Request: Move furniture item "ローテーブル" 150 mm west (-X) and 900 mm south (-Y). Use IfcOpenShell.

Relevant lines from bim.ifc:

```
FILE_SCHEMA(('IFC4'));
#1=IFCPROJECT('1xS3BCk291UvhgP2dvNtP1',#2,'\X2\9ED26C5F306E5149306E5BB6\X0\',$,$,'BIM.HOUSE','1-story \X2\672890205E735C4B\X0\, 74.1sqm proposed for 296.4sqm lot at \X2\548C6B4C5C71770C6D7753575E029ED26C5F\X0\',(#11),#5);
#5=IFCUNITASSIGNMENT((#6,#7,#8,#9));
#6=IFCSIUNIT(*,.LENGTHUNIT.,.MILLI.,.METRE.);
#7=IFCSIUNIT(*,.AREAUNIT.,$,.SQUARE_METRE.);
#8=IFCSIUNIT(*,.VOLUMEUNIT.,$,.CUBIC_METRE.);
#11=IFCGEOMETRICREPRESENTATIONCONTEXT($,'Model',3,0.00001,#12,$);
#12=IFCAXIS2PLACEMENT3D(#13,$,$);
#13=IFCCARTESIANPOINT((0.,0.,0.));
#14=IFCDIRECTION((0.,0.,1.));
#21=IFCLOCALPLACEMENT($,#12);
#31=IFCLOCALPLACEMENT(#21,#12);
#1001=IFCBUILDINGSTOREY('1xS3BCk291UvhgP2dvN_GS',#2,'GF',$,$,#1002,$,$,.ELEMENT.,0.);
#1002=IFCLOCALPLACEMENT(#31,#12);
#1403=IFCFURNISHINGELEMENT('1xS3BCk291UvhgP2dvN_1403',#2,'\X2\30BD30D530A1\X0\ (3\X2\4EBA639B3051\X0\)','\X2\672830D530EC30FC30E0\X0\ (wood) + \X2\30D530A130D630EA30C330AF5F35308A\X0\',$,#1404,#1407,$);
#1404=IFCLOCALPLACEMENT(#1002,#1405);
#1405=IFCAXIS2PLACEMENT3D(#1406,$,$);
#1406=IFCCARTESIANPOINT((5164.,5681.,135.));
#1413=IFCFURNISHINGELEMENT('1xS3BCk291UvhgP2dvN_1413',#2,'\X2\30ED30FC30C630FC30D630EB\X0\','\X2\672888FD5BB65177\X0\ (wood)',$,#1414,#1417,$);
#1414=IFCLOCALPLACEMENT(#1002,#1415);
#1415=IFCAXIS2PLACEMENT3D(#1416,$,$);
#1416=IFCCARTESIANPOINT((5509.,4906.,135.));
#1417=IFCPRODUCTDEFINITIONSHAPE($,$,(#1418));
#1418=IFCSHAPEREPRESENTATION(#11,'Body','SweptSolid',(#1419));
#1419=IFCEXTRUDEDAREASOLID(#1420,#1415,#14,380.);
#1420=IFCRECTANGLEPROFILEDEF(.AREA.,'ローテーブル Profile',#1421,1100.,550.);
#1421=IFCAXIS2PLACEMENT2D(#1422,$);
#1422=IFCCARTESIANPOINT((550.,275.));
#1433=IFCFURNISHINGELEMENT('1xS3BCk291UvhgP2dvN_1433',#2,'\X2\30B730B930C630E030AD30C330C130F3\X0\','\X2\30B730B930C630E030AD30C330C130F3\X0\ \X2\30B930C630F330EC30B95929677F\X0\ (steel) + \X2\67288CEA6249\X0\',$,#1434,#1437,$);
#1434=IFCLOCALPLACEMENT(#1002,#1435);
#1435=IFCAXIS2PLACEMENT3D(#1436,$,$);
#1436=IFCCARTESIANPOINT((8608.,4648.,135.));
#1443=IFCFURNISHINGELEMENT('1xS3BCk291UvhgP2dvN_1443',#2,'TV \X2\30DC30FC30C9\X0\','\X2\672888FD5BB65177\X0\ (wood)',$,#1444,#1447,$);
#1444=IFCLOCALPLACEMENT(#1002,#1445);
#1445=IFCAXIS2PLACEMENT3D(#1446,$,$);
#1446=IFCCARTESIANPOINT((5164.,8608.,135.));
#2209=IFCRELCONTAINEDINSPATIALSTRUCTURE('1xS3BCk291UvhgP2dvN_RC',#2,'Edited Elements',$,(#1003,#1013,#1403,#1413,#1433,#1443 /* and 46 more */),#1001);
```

```python
import ifcopenshell
import ifcopenshell.api.geometry
import ifcopenshell.util.placement

model = ifcopenshell.open("bim.ifc")

item = model.by_guid("1xS3BCk291UvhgP2dvN_1413")
matrix = ifcopenshell.util.placement.get_local_placement(item.ObjectPlacement)
matrix[0, 3] -= 150.0
matrix[1, 3] -= 900.0
ifcopenshell.api.geometry.edit_object_placement(model, product=item, matrix=matrix, is_si=False)

print(ifcopenshell.util.placement.get_local_placement(item.ObjectPlacement).round(3) + 0.0)

model.write("bim_updated.ifc")
```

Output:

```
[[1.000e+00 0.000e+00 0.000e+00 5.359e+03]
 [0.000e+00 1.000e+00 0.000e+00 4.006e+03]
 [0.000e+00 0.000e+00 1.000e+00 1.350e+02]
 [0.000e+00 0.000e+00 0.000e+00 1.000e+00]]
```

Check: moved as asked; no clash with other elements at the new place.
